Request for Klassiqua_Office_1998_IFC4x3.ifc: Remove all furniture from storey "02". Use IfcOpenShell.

First a look at what the model holds.

```python
import ifcopenshell
import ifcopenshell.util.element

model = ifcopenshell.open("Klassiqua_Office_1998_IFC4x3.ifc")
print(model.schema)
storey = next(s for s in model.by_type("IfcBuildingStorey") if s.Name == "02")
furniture = [e for e in ifcopenshell.util.element.get_decomposition(storey) if e.is_a("IfcFurnishingElement")]
seen = {}
for e in furniture:
    element_type = ifcopenshell.util.element.get_type(e)
    name = element_type.Name if element_type not in (None, e) else None
    seen[name] = seen.get(name, 0) + 1
for name, count in sorted(seen.items(), key=str):
    print(count, "x", name)
```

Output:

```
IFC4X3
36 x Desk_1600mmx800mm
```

```python
import ifcopenshell
import ifcopenshell.api.root
import ifcopenshell.util.element

model = ifcopenshell.open("Klassiqua_Office_1998_IFC4x3.ifc")

storey = next(s for s in model.by_type("IfcBuildingStorey") if s.Name == "02")
furniture = [e for e in ifcopenshell.util.element.get_decomposition(storey) if e.is_a("IfcFurnishingElement")]

for e in furniture:
    ifcopenshell.api.root.remove_product(model, product=e)
print(len(furniture), "removed")

model.write("Klassiqua_Office_1998_IFC4x3_v2.ifc")
```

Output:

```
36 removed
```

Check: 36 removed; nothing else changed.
